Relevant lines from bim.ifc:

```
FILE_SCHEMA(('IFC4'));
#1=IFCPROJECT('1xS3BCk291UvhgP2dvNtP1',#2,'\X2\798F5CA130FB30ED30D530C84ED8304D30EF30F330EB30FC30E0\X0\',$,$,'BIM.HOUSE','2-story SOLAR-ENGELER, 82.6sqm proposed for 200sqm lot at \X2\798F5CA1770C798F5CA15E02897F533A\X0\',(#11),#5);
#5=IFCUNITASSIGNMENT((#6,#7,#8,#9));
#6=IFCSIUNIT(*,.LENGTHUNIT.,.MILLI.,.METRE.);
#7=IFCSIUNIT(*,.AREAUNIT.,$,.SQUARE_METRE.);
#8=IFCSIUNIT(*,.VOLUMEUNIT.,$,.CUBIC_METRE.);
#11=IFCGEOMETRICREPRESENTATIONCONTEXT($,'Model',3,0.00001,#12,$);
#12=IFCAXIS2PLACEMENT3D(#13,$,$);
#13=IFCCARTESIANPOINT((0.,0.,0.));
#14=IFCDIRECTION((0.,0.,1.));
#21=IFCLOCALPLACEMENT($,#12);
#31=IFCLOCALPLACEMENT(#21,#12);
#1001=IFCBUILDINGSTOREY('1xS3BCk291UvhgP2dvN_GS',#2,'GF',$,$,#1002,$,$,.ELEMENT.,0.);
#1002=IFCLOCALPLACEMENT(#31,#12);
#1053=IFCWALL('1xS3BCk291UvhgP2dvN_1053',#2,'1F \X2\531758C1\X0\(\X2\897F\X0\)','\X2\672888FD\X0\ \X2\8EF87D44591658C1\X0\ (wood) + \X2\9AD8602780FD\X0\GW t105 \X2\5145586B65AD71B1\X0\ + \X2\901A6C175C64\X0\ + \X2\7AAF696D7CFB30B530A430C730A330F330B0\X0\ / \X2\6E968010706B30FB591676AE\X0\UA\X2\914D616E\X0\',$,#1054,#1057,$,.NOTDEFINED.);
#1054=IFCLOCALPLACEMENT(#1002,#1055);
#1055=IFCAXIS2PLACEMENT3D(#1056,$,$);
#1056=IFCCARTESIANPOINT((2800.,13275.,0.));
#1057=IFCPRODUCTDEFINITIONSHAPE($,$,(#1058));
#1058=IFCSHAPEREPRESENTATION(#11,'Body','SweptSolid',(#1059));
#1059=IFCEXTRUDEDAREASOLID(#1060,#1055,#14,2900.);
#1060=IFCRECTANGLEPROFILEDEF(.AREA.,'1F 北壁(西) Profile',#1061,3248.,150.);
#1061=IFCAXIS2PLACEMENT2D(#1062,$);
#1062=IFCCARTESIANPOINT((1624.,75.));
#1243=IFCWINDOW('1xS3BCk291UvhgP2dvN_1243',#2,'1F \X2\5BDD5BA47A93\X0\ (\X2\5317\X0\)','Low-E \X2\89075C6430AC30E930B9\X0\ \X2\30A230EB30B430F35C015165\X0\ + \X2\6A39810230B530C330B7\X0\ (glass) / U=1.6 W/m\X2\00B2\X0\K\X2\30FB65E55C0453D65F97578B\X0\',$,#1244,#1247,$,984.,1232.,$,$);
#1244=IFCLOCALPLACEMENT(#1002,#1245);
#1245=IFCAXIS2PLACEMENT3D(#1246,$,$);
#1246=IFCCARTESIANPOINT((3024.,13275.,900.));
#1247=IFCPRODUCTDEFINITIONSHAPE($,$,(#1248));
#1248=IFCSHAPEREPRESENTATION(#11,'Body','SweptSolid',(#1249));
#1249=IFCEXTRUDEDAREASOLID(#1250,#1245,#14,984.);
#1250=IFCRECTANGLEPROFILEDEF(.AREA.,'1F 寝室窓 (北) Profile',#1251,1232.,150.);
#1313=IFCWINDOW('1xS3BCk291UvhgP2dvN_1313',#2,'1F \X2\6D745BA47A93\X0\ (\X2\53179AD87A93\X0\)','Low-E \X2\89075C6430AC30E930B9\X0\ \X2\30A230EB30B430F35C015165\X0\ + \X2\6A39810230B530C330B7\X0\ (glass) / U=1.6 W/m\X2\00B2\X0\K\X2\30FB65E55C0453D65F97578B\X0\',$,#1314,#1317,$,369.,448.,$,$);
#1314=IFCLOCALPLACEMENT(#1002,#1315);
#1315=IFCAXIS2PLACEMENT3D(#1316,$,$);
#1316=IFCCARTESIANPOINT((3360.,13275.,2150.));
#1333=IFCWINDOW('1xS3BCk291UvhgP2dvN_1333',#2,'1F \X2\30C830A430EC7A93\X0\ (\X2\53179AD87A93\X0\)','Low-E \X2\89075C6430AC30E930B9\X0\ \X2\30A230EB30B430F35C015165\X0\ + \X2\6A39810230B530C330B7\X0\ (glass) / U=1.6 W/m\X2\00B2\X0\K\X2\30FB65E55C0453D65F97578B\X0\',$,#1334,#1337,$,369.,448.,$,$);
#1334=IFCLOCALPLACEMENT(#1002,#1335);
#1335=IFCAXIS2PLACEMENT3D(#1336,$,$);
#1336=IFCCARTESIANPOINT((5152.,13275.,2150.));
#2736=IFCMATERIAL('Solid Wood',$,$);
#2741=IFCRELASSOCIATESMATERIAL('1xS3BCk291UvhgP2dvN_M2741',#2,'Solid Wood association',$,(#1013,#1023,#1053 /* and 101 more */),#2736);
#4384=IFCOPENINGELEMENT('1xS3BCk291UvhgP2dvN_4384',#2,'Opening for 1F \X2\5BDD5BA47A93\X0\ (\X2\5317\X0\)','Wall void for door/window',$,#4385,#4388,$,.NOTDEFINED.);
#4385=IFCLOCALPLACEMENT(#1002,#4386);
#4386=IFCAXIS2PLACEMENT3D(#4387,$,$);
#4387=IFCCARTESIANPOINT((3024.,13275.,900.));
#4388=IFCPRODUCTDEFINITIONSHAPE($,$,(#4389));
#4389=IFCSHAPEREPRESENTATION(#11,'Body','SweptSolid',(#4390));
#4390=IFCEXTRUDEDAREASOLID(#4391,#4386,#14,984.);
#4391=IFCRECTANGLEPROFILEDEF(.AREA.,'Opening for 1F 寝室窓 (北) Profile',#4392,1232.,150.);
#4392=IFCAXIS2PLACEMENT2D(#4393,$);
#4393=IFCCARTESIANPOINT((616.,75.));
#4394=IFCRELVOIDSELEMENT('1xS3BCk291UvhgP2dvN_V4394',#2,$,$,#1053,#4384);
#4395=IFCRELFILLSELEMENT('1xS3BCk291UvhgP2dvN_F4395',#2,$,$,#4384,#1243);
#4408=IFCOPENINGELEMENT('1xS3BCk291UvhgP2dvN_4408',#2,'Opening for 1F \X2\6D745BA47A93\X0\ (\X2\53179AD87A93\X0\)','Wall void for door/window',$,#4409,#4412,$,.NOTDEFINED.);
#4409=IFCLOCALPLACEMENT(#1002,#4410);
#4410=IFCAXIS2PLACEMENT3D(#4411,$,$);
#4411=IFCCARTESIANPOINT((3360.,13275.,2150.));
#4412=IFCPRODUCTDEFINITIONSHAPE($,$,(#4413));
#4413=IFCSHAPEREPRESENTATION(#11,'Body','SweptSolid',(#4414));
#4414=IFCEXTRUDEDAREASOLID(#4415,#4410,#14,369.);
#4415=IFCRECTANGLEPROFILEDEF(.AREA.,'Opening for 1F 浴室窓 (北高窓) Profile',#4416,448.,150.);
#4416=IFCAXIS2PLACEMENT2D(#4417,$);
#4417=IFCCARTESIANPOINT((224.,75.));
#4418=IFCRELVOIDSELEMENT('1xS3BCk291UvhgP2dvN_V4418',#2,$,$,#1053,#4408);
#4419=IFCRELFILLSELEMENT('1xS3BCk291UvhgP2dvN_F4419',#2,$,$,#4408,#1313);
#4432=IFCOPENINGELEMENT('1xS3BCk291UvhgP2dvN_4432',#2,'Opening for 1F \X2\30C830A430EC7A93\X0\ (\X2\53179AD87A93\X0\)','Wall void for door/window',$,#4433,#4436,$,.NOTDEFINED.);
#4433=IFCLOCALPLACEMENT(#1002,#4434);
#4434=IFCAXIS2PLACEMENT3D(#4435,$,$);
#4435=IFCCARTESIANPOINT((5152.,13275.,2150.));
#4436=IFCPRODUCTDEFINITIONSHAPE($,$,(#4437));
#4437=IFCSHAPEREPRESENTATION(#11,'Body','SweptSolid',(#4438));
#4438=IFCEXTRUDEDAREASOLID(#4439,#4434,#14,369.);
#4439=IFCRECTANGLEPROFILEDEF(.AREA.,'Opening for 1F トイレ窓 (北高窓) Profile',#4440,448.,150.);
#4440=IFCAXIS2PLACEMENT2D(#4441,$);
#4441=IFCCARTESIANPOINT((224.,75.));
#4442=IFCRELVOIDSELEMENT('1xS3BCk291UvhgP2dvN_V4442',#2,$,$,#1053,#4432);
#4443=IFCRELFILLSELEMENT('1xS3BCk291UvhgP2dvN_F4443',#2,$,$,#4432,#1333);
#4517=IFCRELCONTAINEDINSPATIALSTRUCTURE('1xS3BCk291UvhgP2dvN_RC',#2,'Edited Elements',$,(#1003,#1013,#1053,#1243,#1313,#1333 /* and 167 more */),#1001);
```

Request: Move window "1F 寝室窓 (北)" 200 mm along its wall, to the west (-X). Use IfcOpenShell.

```python
import ifcopenshell
import ifcopenshell.api.geometry
import ifcopenshell.util.placement
import ifcopenshell.util.unit

model = ifcopenshell.open("bim.ifc")
unit_scale = ifcopenshell.util.unit.calculate_unit_scale(model)

window = model.by_id(1243)
opening = window.FillsVoids[0].RelatingOpeningElement
wall = opening.VoidsElements[0].RelatingBuildingElement

wall_matrix = ifcopenshell.util.placement.get_local_placement(wall.ObjectPlacement)
shift = wall_matrix[:3, 0] * -0.2 / unit_scale
before = ifcopenshell.util.placement.get_local_placement(window.ObjectPlacement)[:3, 3].copy()

# The window is not placed relative to its opening, so move both.
for product in (opening, window):
    matrix = ifcopenshell.util.placement.get_local_placement(product.ObjectPlacement)
    matrix[:3, 3] += shift
    ifcopenshell.api.geometry.edit_object_placement(model, product=product, matrix=matrix, is_si=False)

after = ifcopenshell.util.placement.get_local_placement(window.ObjectPlacement)[:3, 3]
print("window moved by", (after - before).round(3) + 0.0)

model.write("bim-out.ifc")
```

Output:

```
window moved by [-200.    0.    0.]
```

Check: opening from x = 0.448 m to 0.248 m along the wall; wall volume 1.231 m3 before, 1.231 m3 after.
